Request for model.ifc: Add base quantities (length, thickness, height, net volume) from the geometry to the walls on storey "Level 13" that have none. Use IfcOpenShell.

First a look at what the model holds.

```python
import ifcopenshell
import ifcopenshell.util.element
import ifcopenshell.util.unit

model = ifcopenshell.open("model.ifc")
print(model.schema)
for unit_type in ("LENGTHUNIT", "AREAUNIT", "VOLUMEUNIT"):
    print(unit_type, ifcopenshell.util.unit.calculate_unit_scale(model, unit_type))
storey = next(s for s in model.by_type("IfcBuildingStorey") if s.Name == "Level 13")
walls = [e for e in ifcopenshell.util.element.get_decomposition(storey) if e.is_a("IfcWall")]
for e in sorted(walls, key=lambda e: e.id()):
    print(e.id(), e.is_a(), e.Name, list(ifcopenshell.util.element.get_psets(e, qtos_only=True)), sep=" | ")
```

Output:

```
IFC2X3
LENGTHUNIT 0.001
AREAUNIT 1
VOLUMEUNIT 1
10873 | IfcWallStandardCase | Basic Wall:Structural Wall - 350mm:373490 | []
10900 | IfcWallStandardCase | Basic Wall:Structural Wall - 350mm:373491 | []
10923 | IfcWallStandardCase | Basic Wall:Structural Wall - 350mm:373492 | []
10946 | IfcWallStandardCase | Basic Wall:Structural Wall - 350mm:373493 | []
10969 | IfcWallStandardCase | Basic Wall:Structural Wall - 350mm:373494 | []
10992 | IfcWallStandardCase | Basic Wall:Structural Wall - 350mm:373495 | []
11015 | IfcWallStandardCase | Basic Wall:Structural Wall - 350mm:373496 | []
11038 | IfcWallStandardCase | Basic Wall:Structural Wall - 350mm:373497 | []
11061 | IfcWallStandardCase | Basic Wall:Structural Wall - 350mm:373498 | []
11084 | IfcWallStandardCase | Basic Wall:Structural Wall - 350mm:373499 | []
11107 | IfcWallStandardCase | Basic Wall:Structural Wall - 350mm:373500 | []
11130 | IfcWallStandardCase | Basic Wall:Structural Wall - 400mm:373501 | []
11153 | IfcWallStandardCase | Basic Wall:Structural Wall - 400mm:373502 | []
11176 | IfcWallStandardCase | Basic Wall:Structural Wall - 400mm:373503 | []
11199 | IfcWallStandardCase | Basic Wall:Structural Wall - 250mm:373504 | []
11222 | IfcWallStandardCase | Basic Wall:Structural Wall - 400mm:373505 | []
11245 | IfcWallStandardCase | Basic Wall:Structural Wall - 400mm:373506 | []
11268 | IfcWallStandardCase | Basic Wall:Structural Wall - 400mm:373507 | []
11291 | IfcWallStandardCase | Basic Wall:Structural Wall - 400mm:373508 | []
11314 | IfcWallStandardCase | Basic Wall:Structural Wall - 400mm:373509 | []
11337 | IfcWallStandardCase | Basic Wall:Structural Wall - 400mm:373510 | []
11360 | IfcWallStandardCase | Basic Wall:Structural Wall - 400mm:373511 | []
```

```python
import ifcopenshell
import ifcopenshell.api.pset
import ifcopenshell.geom
import ifcopenshell.util.element
import ifcopenshell.util.shape
import ifcopenshell.util.unit

model = ifcopenshell.open("model.ifc")
unit_scale = ifcopenshell.util.unit.calculate_unit_scale(model)
volume_scale = ifcopenshell.util.unit.calculate_unit_scale(model, "VOLUMEUNIT")
settings = ifcopenshell.geom.settings()

storey = next(s for s in model.by_type("IfcBuildingStorey") if s.Name == "Level 13")
walls = [e for e in ifcopenshell.util.element.get_decomposition(storey) if e.is_a("IfcWall")]

for e in sorted(walls, key=lambda e: e.id()):
    if ifcopenshell.util.element.get_psets(e, qtos_only=True, should_inherit=False):
        continue
    # Geometry comes back in metres, in the element's own axes.
    shape = ifcopenshell.geom.create_shape(settings, e)
    values = {
        "Length": ifcopenshell.util.shape.get_x(shape.geometry) / unit_scale,
        "Width": ifcopenshell.util.shape.get_y(shape.geometry) / unit_scale,
        "Height": ifcopenshell.util.shape.get_z(shape.geometry) / unit_scale,
        "NetVolume": ifcopenshell.util.shape.get_volume(shape.geometry) / volume_scale,
    }
    qto = ifcopenshell.api.pset.add_qto(model, product=e, name="BaseQuantities")
    ifcopenshell.api.pset.edit_qto(model, qto=qto, properties=values)
    print(e.id(), {k: round(v, 3) for k, v in values.items()})

model.write("model_updated.ifc")
```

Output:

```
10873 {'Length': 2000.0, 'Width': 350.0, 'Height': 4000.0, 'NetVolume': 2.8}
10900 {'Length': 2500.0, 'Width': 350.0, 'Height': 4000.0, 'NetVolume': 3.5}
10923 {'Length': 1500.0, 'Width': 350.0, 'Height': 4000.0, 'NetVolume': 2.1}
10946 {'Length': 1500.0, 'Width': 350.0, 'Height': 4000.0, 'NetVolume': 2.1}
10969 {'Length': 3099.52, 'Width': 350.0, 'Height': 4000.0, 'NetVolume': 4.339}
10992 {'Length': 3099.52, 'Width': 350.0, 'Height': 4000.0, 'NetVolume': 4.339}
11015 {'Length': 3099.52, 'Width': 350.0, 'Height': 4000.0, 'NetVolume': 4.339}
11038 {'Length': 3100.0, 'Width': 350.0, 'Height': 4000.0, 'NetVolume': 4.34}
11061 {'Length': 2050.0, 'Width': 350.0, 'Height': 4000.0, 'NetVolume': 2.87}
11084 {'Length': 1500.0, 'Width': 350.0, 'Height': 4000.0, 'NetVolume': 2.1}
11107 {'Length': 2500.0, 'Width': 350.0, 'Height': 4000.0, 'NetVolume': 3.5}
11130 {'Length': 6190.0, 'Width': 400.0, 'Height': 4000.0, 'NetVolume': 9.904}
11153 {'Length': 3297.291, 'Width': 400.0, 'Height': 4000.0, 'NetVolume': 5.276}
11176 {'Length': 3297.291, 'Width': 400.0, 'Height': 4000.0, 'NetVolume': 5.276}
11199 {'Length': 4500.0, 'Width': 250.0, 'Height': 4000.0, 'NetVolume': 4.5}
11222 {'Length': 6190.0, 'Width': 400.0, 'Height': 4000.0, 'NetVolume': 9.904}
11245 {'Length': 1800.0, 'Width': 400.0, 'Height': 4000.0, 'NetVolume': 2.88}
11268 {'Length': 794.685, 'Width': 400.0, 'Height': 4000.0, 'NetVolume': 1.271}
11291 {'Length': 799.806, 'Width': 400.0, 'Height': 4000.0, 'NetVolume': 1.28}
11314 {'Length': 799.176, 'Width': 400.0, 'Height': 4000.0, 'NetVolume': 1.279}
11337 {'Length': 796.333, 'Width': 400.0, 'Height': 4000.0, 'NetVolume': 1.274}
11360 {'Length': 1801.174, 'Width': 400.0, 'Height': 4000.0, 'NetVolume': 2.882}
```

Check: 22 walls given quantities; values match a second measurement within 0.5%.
